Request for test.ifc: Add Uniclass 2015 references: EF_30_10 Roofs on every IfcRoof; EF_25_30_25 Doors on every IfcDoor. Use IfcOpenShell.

First a look at what the model holds.

```python
import ifcopenshell

model = ifcopenshell.open("test.ifc")
print(model.schema)
print("classifications:", [c.Name for c in model.by_type("IfcClassification")])
for ifc_class in ("IfcDoor", "IfcRoof", "IfcStair", "IfcWall", "IfcWindow"):
    print(ifc_class, len(model.by_type(ifc_class)))
```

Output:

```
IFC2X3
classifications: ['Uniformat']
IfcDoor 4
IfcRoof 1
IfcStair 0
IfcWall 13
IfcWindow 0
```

```python
import ifcopenshell
import ifcopenshell.api.classification

model = ifcopenshell.open("test.ifc")

# IFC2X3 requires Source and Edition and has no link from the project to the system.
system = model.create_entity("IfcClassification", Source="NBS", Edition="2015", Name="Uniclass 2015")

codes = {
    "IfcRoof": ("EF_30_10", "Roofs"),
    "IfcDoor": ("EF_25_30_25", "Doors"),
}
for ifc_class, (code, name) in codes.items():
    products = model.by_type(ifc_class)
    ifcopenshell.api.classification.add_reference(
        model, products=products, classification=system, identification=code, name=name
    )
    print(code, len(products))

model.write("test_edited.ifc")
```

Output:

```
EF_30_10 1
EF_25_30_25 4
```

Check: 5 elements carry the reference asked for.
